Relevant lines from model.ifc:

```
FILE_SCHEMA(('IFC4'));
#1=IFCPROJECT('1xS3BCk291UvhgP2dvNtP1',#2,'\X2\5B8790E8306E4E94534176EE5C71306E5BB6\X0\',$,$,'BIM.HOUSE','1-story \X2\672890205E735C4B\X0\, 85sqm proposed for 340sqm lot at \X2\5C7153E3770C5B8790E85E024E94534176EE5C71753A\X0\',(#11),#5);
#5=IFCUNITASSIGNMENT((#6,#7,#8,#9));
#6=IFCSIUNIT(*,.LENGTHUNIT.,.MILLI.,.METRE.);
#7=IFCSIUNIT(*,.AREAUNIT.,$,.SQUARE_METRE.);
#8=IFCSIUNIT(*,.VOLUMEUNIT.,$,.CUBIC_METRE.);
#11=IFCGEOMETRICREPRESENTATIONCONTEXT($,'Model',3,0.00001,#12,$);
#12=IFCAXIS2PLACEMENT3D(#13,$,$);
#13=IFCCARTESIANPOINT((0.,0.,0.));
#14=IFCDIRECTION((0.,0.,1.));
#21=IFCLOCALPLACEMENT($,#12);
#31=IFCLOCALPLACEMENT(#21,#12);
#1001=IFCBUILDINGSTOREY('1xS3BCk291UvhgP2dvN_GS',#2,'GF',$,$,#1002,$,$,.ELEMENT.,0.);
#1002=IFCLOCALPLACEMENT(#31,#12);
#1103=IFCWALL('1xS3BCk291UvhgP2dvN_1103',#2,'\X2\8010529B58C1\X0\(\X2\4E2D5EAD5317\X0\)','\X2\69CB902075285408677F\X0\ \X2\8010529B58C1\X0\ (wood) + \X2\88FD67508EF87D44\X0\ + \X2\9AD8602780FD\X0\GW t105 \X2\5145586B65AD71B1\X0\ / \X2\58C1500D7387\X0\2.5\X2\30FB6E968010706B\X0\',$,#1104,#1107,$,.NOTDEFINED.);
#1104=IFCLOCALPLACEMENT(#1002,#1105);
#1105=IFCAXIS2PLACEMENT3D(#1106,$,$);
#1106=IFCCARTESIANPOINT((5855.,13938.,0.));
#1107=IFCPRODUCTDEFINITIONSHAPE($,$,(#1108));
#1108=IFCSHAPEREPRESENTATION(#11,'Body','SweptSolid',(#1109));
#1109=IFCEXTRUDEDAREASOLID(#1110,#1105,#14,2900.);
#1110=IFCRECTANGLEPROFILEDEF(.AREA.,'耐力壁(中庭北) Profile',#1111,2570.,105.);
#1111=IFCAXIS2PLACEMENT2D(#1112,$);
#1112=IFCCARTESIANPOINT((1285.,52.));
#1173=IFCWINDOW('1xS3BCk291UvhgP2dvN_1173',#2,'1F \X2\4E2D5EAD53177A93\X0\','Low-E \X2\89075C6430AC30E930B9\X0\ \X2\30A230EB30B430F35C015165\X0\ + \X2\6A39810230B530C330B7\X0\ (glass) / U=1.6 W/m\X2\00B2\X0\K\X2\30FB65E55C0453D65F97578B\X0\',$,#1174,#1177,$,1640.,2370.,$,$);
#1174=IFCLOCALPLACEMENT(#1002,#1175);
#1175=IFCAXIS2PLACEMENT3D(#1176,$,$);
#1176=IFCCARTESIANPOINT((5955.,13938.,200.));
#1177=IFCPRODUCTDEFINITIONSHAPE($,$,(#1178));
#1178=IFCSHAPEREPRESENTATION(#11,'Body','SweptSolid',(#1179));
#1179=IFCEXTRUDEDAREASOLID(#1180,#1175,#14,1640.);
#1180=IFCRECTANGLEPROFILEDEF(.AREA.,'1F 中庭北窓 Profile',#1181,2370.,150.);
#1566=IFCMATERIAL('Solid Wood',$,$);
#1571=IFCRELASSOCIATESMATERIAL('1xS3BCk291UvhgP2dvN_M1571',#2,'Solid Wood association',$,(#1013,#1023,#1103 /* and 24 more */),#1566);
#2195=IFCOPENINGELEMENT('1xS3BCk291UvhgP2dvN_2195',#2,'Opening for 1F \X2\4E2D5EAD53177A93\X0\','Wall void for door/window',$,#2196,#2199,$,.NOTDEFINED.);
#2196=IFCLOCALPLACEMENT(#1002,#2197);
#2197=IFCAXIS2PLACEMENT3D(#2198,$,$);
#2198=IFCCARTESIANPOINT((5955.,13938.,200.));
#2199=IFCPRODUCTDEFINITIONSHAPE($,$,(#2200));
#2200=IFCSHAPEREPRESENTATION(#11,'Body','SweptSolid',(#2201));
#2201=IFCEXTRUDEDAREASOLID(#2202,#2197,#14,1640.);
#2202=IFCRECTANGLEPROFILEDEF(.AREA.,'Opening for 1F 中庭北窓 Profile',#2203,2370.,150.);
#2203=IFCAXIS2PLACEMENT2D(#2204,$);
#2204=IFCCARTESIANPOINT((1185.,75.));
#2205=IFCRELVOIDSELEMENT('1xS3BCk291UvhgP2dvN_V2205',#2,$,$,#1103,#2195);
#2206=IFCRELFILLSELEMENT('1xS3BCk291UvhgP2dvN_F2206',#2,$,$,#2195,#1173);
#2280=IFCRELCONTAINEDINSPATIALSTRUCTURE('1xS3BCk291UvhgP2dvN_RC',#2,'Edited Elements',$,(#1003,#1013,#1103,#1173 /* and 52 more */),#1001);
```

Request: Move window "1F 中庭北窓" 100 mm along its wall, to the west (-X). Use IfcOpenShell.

```python
import ifcopenshell
import ifcopenshell.api.geometry
import ifcopenshell.util.placement
import ifcopenshell.util.unit

model = ifcopenshell.open("model.ifc")
unit_scale = ifcopenshell.util.unit.calculate_unit_scale(model)

window = model.by_guid("1xS3BCk291UvhgP2dvN_1173")
opening = window.FillsVoids[0].RelatingOpeningElement
wall = opening.VoidsElements[0].RelatingBuildingElement

wall_matrix = ifcopenshell.util.placement.get_local_placement(wall.ObjectPlacement)
shift = wall_matrix[:3, 0] * -0.1 / unit_scale
before = ifcopenshell.util.placement.get_local_placement(window.ObjectPlacement)[:3, 3].copy()

# The window is not placed relative to its opening, so move both.
for product in (opening, window):
    matrix = ifcopenshell.util.placement.get_local_placement(product.ObjectPlacement)
    matrix[:3, 3] += shift
    ifcopenshell.api.geometry.edit_object_placement(model, product=product, matrix=matrix, is_si=False)

after = ifcopenshell.util.placement.get_local_placement(window.ObjectPlacement)[:3, 3]
print("window moved by", (after - before).round(3) + 0.0)

model.write("model_updated.ifc")
```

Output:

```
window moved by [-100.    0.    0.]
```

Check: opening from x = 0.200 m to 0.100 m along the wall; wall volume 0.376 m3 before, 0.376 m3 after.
